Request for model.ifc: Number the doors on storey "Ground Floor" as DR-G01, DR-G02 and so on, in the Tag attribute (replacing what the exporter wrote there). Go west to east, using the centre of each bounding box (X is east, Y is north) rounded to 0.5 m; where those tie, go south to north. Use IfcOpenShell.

First a look at what the model holds.

```python
import ifcopenshell
import ifcopenshell.util.element
import ifcopenshell.util.placement

model = ifcopenshell.open("model.ifc")
print(model.schema)
storey = next(s for s in model.by_type("IfcBuildingStorey") if s.Name == "Ground Floor")
doors = [e for e in ifcopenshell.util.element.get_decomposition(storey) if e.is_a("IfcDoor")]
for e in sorted(doors, key=lambda e: e.id()):
    origin = ifcopenshell.util.placement.get_local_placement(e.ObjectPlacement)[:3, 3]
    print(e.id(), e.Tag, e.Name, origin.round(2) + 0.0, sep=" | ")
```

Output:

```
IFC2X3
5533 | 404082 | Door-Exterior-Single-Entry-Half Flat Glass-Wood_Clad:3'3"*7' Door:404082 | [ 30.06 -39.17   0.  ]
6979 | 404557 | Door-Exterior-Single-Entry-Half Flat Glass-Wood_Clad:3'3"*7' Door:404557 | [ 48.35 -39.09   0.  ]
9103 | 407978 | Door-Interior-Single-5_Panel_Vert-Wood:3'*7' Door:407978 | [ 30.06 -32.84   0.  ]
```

```python
import ifcopenshell
import ifcopenshell.geom
import ifcopenshell.util.element
import ifcopenshell.util.shape

model = ifcopenshell.open("model.ifc")
settings = ifcopenshell.geom.settings()
settings.set("use-world-coords", True)


def centre(element):
    shape = ifcopenshell.geom.create_shape(settings, element)
    return ifcopenshell.util.shape.get_bbox_centroid(shape.geometry)


storey = next(s for s in model.by_type("IfcBuildingStorey") if s.Name == "Ground Floor")
doors = [e for e in ifcopenshell.util.element.get_decomposition(storey) if e.is_a("IfcDoor")]

# Insertion points can sit at a corner or the storey origin, so sort by the geometry (in metres).
centres = {e: centre(e) for e in doors}
doors.sort(key=lambda e: (round(centres[e][0] / 0.5), centres[e][1]))

for i, e in enumerate(doors, start=1):
    number = f"DR-G{i:02d}"
    e.Tag = number
    print(e.id(), number)

model.write("model-out.ifc")
```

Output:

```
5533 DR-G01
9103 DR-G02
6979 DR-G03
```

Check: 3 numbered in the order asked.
